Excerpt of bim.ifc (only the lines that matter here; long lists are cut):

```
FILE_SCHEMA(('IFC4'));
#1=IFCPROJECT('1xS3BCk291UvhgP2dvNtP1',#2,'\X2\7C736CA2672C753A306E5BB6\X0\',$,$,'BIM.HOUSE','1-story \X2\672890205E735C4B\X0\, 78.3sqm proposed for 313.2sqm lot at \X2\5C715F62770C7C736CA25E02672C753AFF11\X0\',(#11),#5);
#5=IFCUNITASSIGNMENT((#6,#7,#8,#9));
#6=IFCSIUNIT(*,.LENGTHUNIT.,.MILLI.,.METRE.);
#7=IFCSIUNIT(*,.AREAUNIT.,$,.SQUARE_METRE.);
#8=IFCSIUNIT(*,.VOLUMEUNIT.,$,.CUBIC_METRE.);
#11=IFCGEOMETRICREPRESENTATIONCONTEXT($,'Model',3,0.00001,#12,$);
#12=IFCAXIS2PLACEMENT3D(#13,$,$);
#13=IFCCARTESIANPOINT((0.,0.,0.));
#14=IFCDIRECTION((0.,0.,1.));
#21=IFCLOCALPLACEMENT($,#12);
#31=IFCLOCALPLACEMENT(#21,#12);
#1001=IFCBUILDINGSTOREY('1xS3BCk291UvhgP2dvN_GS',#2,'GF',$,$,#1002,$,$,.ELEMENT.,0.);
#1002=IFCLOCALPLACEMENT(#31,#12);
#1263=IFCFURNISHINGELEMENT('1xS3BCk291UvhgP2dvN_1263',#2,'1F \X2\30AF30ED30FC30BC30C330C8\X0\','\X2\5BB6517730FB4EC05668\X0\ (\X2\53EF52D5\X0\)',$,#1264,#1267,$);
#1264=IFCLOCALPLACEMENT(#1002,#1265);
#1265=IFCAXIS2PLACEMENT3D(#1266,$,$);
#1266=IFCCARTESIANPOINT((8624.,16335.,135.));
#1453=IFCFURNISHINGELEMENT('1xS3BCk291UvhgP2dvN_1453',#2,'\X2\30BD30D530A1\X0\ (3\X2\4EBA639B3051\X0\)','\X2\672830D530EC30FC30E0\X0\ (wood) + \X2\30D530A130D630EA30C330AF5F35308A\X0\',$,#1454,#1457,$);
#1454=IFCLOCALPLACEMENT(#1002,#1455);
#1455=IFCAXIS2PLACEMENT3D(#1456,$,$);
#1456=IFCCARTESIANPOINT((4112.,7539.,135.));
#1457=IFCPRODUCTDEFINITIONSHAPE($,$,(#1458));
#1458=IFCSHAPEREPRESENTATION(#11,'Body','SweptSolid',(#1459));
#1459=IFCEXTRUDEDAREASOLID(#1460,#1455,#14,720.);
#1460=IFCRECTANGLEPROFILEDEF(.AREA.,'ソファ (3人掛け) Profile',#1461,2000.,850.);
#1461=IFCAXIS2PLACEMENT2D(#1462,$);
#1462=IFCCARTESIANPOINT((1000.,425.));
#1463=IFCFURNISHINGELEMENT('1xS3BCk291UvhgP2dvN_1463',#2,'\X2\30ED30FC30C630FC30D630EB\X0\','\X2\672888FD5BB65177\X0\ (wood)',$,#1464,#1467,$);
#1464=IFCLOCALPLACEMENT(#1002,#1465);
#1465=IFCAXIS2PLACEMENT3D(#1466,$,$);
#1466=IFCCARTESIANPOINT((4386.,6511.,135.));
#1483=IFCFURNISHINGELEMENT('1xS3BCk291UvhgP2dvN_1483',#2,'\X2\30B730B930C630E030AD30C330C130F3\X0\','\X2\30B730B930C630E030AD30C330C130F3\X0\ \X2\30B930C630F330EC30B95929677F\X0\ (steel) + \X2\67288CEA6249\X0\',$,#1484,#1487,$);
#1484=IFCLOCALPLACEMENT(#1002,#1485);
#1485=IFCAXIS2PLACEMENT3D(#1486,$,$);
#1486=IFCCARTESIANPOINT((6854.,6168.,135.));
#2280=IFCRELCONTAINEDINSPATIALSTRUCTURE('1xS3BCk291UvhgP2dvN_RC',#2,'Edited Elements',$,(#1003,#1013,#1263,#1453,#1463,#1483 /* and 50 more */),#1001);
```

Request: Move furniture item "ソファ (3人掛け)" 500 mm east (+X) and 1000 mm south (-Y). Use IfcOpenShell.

```python
import ifcopenshell
import ifcopenshell.api.geometry
import ifcopenshell.util.placement
import ifcopenshell.util.unit

model = ifcopenshell.open("bim.ifc")
unit_scale = ifcopenshell.util.unit.calculate_unit_scale(model)

item = model.by_id(1453)
matrix = ifcopenshell.util.placement.get_local_placement(item.ObjectPlacement)
matrix[0, 3] += 0.5 / unit_scale
matrix[1, 3] -= 1 / unit_scale
ifcopenshell.api.geometry.edit_object_placement(model, product=item, matrix=matrix, is_si=False)

print(ifcopenshell.util.placement.get_local_placement(item.ObjectPlacement).round(3) + 0.0)

model.write("bim_v2.ifc")
```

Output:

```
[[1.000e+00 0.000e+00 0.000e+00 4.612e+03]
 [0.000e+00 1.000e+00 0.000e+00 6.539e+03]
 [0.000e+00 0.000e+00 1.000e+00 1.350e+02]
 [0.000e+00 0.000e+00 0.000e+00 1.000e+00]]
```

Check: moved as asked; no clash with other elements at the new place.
